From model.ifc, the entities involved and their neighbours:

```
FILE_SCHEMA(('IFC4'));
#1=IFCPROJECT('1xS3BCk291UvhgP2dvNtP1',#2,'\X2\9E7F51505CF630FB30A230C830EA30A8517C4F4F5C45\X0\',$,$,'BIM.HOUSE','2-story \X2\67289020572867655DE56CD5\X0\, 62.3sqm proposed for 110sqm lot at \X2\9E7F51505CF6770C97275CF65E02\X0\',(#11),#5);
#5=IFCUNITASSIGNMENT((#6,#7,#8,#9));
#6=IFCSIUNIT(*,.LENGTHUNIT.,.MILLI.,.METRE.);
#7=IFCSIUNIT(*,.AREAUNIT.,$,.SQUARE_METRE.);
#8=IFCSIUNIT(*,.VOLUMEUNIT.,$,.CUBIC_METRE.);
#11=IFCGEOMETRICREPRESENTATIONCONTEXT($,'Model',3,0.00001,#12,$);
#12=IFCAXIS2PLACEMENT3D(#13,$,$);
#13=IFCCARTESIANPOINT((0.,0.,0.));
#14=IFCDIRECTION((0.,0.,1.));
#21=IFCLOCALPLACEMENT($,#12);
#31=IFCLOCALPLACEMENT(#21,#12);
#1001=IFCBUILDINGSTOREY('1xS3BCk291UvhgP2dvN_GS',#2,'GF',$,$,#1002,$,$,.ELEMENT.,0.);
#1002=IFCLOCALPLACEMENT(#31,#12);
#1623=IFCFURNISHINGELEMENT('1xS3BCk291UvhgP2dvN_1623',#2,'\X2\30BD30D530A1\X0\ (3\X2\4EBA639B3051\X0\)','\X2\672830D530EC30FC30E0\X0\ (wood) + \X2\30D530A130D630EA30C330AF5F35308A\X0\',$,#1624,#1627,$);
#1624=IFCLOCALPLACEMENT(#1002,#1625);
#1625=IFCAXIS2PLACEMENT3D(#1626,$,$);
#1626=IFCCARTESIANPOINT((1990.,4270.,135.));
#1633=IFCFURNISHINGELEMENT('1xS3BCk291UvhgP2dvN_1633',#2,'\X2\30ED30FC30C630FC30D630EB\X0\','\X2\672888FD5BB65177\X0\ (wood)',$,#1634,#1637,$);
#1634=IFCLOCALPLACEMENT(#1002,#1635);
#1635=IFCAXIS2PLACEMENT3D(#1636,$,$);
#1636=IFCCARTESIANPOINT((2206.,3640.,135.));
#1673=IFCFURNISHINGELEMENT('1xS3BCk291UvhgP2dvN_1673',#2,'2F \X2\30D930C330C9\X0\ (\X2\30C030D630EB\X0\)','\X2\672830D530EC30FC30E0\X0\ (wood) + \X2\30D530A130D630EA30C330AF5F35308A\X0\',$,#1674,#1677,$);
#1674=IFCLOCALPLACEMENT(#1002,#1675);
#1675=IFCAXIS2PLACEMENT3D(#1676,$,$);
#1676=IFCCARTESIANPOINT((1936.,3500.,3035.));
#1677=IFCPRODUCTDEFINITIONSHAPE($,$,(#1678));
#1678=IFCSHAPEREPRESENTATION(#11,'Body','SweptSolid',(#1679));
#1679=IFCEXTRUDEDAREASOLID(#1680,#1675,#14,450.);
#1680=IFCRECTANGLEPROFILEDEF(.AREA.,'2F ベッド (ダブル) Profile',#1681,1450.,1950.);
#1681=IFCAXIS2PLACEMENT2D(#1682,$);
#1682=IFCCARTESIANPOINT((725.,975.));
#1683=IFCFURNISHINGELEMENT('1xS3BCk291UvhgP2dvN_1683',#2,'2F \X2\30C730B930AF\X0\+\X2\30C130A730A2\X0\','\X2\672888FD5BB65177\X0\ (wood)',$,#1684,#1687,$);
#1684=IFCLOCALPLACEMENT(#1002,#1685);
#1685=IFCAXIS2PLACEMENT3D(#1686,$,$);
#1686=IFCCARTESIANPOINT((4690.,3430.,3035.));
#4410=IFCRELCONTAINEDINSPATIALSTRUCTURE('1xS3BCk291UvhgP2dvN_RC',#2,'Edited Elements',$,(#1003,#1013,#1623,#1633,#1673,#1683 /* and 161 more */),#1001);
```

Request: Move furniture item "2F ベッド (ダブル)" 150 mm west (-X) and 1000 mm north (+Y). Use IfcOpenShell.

```python
import ifcopenshell
import ifcopenshell.api.geometry
import ifcopenshell.util.placement

model = ifcopenshell.open("model.ifc")

item = model.by_guid("1xS3BCk291UvhgP2dvN_1673")
matrix = ifcopenshell.util.placement.get_local_placement(item.ObjectPlacement)
matrix[0, 3] -= 150.0
matrix[1, 3] += 1000.0
ifcopenshell.api.geometry.edit_object_placement(model, product=item, matrix=matrix, is_si=False)

print(ifcopenshell.util.placement.get_local_placement(item.ObjectPlacement).round(3) + 0.0)

model.write("model_updated.ifc")
```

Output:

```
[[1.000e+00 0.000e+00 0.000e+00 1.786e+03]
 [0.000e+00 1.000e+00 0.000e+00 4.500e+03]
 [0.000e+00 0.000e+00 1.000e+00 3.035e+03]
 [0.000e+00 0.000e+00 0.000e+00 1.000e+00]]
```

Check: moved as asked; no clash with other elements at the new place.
